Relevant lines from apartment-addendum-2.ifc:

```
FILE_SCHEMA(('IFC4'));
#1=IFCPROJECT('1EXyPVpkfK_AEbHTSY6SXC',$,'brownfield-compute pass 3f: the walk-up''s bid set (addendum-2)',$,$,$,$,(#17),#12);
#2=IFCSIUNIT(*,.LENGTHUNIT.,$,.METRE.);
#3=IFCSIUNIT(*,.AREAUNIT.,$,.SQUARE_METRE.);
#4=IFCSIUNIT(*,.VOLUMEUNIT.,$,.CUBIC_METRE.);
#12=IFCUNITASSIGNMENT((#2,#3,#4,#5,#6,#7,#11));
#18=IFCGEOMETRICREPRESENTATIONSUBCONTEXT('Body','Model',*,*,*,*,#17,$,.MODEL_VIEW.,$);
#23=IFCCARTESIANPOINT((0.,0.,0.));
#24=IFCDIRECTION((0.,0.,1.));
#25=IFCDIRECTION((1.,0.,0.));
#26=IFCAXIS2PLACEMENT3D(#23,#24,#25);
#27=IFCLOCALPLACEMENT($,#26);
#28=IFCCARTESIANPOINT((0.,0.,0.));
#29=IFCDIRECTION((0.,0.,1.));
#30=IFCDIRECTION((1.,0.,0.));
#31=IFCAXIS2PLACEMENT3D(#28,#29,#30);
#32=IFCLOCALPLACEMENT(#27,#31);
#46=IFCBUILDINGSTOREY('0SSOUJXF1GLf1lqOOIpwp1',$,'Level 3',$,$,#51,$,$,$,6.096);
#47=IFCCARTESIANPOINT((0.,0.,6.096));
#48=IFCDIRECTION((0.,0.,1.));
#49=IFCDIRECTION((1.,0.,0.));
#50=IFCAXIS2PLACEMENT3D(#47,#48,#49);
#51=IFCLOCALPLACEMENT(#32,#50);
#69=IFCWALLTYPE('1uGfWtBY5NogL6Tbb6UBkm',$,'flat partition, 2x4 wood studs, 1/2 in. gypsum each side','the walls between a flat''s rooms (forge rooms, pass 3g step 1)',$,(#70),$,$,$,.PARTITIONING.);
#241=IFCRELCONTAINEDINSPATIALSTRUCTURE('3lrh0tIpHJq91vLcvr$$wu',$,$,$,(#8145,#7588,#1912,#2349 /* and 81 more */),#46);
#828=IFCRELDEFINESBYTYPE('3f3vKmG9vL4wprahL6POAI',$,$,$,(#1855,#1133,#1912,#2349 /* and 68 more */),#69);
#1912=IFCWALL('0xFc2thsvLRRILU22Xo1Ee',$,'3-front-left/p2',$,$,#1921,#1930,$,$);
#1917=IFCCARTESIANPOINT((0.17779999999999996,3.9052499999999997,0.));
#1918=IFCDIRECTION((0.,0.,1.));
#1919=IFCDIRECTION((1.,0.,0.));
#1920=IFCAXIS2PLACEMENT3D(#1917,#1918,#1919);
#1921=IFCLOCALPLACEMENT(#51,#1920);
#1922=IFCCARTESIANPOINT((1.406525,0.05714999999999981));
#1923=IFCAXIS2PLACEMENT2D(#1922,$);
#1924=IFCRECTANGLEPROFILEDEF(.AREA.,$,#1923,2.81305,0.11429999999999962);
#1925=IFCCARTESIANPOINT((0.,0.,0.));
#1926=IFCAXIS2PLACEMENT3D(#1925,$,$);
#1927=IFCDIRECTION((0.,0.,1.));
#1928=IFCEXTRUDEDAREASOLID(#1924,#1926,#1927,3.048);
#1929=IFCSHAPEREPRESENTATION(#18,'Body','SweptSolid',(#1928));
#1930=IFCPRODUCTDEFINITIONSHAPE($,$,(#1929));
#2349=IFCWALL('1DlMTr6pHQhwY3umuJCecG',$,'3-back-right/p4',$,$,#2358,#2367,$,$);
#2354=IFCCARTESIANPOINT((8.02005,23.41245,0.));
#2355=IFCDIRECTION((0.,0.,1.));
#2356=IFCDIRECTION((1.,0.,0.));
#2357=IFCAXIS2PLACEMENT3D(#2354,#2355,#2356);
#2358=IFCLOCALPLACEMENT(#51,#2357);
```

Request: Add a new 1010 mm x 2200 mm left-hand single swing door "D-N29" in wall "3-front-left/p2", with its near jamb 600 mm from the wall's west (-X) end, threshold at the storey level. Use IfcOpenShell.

```python
import numpy as np
import ifcopenshell
import ifcopenshell.api.feature
import ifcopenshell.api.geometry
import ifcopenshell.api.root
import ifcopenshell.api.spatial
import ifcopenshell.geom
import ifcopenshell.util.element
import ifcopenshell.util.placement
import ifcopenshell.util.representation
import ifcopenshell.util.shape
import ifcopenshell.util.unit

model = ifcopenshell.open("apartment-addendum-2.ifc")
unit_scale = ifcopenshell.util.unit.calculate_unit_scale(model)
settings = ifcopenshell.geom.settings()


def volume(element):
    """Net volume in cubic metres, openings subtracted."""
    shape = ifcopenshell.geom.create_shape(settings, element)
    return ifcopenshell.util.shape.get_volume(shape.geometry)


wall = model.by_id(1912)
storey = ifcopenshell.util.element.get_container(wall, ifc_class="IfcBuildingStorey")
context = ifcopenshell.util.representation.get_context(model, "Model", "Body", "MODEL_VIEW")
before = volume(wall)

width, height, from_end, sill = 1.01, 2.2, 0.6, 0.0  # metres

# The wall runs along its own X axis, and the end named is its -X end.
wall_shape = ifcopenshell.geom.create_shape(settings, wall)
x, y, z = ifcopenshell.util.shape.get_vertices(wall_shape.geometry).T
start = x.min() + from_end
face, thickness = float(y.min()), float(y.max() - y.min())
wall_matrix = ifcopenshell.util.placement.get_local_placement(wall.ObjectPlacement)
level = ifcopenshell.util.placement.get_local_placement(storey.ObjectPlacement)[2, 3]


def in_wall(x, y):
    """Placement at x, y metres in the wall's axes, at sill height."""
    matrix = wall_matrix.copy()
    matrix[:, 3] = wall_matrix @ np.array([x / unit_scale, y / unit_scale, 0.0, 1.0])
    matrix[2, 3] = level + sill / unit_scale
    return matrix


# Opening: a box that overshoots both wall faces by 50 mm.
opening = ifcopenshell.api.root.create_entity(model, ifc_class="IfcOpeningElement", predefined_type="OPENING")
box = ifcopenshell.api.geometry.add_wall_representation(
    model, context=context, length=width, height=height, thickness=thickness + 0.1
)
ifcopenshell.api.geometry.assign_representation(model, product=opening, representation=box)
ifcopenshell.api.geometry.edit_object_placement(model, product=opening, matrix=in_wall(start, face - 0.05), is_si=False)
ifcopenshell.api.feature.add_feature(model, feature=opening, element=wall)

door = ifcopenshell.api.root.create_entity(model, ifc_class="IfcDoor", name="D-N29", predefined_type="DOOR")
door.OverallWidth, door.OverallHeight = width / unit_scale, height / unit_scale
door.OperationType = "SINGLE_SWING_LEFT"
body = ifcopenshell.api.geometry.add_door_representation(
    model,
    context=context,
    overall_width=door.OverallWidth,
    overall_height=door.OverallHeight,
    operation_type="SINGLE_SWING_LEFT",
    lining_properties={"LiningDepth": thickness / unit_scale, "ThresholdDepth": thickness / unit_scale},
)
ifcopenshell.api.geometry.assign_representation(model, product=door, representation=body)
ifcopenshell.api.spatial.assign_container(model, products=[door], relating_structure=storey)
ifcopenshell.api.feature.add_filling(model, opening=opening, element=door)

# The lining spans the wall, so the door starts at the wall face.
ifcopenshell.api.geometry.edit_object_placement(model, product=door, matrix=in_wall(start, face), is_si=False)

after = volume(wall)

print(f"wall volume {before:.3f} -> {after:.3f} m3")

model.write("apartment-addendum-2-out.ifc")
```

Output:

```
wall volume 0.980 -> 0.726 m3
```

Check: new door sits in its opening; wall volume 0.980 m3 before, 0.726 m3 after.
